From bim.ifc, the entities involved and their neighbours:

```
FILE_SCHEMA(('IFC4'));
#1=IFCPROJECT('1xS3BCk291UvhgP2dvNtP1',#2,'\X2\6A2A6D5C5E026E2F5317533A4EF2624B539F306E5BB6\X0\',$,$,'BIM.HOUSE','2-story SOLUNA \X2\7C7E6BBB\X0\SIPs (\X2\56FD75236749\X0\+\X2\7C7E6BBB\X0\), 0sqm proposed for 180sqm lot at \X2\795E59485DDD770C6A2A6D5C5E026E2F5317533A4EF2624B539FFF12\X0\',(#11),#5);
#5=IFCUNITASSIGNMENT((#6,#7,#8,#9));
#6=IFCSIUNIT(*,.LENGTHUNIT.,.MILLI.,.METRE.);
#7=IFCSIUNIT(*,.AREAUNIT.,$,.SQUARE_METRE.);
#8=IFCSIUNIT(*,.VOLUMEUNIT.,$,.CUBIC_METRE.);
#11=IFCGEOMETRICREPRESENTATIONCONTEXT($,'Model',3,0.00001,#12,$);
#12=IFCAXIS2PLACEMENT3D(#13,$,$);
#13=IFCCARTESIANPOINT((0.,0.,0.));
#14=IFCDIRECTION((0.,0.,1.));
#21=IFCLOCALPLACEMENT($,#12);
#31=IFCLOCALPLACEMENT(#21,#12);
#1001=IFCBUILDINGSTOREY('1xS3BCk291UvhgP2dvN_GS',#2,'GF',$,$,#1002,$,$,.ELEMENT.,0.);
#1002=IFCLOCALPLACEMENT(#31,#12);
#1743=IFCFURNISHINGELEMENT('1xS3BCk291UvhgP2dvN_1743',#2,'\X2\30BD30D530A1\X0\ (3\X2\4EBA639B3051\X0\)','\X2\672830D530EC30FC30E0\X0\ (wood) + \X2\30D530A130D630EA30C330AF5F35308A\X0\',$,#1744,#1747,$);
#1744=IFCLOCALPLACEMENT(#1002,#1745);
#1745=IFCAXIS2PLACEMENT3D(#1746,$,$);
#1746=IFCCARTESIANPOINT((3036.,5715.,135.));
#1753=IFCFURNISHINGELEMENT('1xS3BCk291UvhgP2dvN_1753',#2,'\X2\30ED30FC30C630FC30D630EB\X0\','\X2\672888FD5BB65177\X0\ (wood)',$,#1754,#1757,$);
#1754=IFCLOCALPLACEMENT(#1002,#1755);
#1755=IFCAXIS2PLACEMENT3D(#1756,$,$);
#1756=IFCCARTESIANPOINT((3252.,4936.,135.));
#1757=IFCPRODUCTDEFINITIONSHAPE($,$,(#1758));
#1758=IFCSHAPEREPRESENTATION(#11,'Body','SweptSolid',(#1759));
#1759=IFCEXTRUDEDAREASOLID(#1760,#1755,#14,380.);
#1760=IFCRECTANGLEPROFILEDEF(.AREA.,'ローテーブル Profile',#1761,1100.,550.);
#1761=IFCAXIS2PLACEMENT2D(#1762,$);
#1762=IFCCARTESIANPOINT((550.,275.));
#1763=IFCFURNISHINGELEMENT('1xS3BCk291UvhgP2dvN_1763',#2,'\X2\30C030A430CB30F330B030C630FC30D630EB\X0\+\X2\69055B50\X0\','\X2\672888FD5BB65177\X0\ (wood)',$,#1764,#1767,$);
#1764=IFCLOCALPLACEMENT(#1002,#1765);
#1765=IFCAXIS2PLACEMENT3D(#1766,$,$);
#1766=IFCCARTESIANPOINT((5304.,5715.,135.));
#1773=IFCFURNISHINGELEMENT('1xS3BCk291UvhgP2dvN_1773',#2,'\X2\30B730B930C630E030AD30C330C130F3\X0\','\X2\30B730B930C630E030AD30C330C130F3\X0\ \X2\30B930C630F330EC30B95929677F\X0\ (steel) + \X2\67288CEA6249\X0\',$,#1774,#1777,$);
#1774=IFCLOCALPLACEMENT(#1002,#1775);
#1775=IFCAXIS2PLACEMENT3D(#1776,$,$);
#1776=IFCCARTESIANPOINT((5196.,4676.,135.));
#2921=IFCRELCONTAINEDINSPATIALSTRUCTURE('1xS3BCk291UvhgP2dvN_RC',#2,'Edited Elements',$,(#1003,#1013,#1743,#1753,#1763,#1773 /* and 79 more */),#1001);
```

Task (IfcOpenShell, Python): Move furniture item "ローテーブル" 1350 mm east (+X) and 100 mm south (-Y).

```python
import ifcopenshell
import ifcopenshell.api.geometry
import ifcopenshell.util.placement
import ifcopenshell.util.unit

model = ifcopenshell.open("bim.ifc")
unit_scale = ifcopenshell.util.unit.calculate_unit_scale(model)

item = model.by_id(1753)
matrix = ifcopenshell.util.placement.get_local_placement(item.ObjectPlacement)
matrix[0, 3] += 1.35 / unit_scale
matrix[1, 3] -= 0.1 / unit_scale
ifcopenshell.api.geometry.edit_object_placement(model, product=item, matrix=matrix, is_si=False)

print(ifcopenshell.util.placement.get_local_placement(item.ObjectPlacement).round(3) + 0.0)

model.write("bim_updated.ifc")
```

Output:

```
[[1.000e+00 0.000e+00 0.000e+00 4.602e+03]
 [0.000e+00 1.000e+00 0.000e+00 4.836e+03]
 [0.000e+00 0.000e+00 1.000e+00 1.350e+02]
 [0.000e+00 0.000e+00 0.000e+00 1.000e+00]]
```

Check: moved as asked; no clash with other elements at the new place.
